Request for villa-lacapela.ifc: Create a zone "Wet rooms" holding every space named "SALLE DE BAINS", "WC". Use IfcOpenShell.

First a look at what the model holds.

```python
import ifcopenshell

model = ifcopenshell.open("villa-lacapela.ifc")
print(model.schema)
seen = {}
for space in model.by_type("IfcSpace"):
    seen[space.LongName] = seen.get(space.LongName, 0) + 1
for name, count in sorted(seen.items(), key=str):
    print(count, "x", name)
print("zones:", [z.Name for z in model.by_type("IfcZone")][:20])
```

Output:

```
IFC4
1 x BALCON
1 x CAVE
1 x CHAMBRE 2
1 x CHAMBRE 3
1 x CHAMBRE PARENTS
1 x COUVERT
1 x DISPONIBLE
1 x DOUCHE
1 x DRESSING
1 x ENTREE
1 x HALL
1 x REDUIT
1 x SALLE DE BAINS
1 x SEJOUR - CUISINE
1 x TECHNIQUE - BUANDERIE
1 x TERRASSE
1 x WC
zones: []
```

```python
import ifcopenshell
import ifcopenshell.api.group
import ifcopenshell.api.root

model = ifcopenshell.open("villa-lacapela.ifc")

names = {"SALLE DE BAINS", "WC"}
spaces = [s for s in model.by_type("IfcSpace") if s.LongName in names]

zone = ifcopenshell.api.root.create_entity(model, ifc_class="IfcZone", name="Wet rooms")
ifcopenshell.api.group.assign_group(model, products=spaces, group=zone)
print(len(spaces), "spaces in", zone.Name)

model.write("villa-lacapela_updated.ifc")
```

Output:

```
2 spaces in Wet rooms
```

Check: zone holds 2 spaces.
